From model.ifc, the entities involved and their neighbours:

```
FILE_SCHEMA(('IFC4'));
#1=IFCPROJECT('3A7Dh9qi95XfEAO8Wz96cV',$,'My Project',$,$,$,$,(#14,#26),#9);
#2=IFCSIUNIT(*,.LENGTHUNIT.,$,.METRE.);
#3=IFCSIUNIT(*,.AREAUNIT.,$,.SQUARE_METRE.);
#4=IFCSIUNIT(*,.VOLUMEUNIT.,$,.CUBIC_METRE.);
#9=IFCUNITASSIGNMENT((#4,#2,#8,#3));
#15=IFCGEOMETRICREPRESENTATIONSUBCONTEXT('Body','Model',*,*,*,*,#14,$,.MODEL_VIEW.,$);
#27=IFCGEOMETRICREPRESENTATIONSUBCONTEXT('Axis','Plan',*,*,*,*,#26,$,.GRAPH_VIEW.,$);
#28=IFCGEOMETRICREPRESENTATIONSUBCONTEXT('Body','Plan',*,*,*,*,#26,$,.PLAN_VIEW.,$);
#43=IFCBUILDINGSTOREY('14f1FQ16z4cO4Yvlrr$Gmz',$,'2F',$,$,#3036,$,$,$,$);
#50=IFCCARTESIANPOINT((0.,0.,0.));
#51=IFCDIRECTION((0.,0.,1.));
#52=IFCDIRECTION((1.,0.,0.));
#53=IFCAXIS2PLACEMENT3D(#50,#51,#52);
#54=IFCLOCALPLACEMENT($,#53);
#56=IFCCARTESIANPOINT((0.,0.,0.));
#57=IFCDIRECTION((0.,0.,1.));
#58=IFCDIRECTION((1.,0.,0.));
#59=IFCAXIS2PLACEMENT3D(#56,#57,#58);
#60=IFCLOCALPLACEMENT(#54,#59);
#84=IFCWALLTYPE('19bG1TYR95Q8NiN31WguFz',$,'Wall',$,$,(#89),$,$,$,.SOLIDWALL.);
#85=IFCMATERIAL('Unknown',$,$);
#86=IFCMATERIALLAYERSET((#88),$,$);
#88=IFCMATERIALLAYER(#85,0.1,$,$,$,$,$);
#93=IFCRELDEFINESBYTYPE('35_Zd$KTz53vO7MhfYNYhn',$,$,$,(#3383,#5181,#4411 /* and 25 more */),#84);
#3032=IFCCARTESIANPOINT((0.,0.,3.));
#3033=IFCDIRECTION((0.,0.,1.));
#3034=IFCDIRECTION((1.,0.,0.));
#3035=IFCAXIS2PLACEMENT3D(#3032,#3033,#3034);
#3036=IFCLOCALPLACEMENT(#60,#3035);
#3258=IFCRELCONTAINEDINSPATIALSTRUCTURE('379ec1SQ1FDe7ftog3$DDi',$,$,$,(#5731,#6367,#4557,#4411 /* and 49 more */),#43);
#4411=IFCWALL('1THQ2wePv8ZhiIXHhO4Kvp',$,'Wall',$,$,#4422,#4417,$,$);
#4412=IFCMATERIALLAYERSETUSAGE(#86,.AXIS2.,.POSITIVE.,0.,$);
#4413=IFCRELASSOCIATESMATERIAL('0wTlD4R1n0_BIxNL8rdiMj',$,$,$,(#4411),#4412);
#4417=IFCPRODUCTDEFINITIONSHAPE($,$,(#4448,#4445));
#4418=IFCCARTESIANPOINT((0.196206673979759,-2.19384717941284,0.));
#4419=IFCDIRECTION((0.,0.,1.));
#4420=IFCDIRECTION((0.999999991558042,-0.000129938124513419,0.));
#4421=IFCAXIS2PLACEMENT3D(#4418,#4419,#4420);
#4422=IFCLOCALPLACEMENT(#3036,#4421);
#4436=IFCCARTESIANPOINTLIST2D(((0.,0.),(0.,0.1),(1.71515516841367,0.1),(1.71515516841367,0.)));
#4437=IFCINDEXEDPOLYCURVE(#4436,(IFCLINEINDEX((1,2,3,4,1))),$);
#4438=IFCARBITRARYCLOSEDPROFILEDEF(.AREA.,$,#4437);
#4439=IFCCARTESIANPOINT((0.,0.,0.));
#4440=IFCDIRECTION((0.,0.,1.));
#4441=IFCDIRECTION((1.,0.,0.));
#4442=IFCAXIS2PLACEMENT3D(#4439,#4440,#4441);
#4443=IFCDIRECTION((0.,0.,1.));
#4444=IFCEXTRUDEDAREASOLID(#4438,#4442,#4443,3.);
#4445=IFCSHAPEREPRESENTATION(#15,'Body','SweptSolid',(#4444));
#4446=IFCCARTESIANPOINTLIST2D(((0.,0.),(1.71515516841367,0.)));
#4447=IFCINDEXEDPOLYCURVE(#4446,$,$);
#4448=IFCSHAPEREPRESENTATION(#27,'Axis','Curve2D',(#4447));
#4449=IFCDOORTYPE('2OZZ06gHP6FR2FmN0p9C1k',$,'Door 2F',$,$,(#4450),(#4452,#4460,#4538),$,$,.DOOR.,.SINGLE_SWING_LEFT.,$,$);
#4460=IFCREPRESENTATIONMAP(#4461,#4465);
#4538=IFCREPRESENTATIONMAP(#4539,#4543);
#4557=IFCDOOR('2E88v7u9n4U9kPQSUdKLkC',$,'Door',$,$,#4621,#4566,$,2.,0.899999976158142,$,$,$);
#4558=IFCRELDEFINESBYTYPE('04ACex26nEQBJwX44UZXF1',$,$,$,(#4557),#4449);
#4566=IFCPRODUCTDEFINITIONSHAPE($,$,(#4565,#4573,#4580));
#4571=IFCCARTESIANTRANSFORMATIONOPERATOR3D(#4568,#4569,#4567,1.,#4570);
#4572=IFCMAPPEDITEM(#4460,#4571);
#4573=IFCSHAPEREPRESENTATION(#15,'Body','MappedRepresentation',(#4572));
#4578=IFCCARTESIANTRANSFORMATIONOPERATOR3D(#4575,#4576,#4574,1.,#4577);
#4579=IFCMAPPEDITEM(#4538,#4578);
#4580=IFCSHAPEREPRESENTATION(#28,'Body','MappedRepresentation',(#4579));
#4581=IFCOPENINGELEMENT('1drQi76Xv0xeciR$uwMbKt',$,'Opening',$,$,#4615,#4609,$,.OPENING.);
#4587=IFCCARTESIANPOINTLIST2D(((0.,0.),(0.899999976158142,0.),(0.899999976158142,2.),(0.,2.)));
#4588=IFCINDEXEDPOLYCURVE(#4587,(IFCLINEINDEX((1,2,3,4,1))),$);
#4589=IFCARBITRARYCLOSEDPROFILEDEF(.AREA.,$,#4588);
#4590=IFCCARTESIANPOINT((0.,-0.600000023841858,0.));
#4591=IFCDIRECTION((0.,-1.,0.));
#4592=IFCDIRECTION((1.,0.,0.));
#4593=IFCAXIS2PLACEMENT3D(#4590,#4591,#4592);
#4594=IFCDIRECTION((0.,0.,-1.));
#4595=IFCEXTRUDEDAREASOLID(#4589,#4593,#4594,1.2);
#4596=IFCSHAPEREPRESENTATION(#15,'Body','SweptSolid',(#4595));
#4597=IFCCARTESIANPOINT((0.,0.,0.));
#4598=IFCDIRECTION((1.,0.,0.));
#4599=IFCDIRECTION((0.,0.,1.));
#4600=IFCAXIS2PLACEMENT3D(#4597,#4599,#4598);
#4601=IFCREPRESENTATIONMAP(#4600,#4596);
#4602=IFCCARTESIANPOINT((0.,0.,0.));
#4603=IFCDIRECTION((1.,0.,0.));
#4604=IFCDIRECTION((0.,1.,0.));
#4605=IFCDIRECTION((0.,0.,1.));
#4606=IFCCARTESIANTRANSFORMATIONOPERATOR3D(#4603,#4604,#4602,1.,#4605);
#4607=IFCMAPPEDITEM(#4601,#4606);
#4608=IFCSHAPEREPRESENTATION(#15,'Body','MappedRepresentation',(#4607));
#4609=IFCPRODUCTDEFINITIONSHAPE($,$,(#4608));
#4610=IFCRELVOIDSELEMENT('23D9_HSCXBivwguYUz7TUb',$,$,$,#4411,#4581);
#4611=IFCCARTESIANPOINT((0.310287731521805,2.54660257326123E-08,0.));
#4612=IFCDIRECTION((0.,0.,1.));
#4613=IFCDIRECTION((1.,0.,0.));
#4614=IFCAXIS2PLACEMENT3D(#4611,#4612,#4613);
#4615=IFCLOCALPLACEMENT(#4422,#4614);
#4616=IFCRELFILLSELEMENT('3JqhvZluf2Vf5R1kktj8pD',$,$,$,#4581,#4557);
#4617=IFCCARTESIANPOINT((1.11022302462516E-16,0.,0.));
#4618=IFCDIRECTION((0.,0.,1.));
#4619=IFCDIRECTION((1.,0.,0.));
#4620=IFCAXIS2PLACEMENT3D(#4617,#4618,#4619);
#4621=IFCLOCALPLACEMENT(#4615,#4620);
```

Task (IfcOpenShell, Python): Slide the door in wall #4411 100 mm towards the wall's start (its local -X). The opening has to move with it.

```python
import ifcopenshell
import ifcopenshell.api.geometry
import ifcopenshell.util.placement

model = ifcopenshell.open("model.ifc")

door = model.by_guid("2E88v7u9n4U9kPQSUdKLkC")
opening = door.FillsVoids[0].RelatingOpeningElement
wall = opening.VoidsElements[0].RelatingBuildingElement

wall_matrix = ifcopenshell.util.placement.get_local_placement(wall.ObjectPlacement)
shift = wall_matrix[:3, 0] * -0.1
before = ifcopenshell.util.placement.get_local_placement(door.ObjectPlacement)[:3, 3].copy()

# The door is placed relative to its opening, so it follows when the opening moves.
matrix = ifcopenshell.util.placement.get_local_placement(opening.ObjectPlacement)
matrix[:3, 3] += shift
ifcopenshell.api.geometry.edit_object_placement(
    model, product=opening, matrix=matrix, is_si=False, should_transform_children=True
)

after = ifcopenshell.util.placement.get_local_placement(door.ObjectPlacement)[:3, 3]
print("door moved by", (after - before).round(3) + 0.0)

model.write("model_v2.ifc")
```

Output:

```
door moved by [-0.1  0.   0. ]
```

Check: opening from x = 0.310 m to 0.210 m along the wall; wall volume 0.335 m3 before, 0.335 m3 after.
